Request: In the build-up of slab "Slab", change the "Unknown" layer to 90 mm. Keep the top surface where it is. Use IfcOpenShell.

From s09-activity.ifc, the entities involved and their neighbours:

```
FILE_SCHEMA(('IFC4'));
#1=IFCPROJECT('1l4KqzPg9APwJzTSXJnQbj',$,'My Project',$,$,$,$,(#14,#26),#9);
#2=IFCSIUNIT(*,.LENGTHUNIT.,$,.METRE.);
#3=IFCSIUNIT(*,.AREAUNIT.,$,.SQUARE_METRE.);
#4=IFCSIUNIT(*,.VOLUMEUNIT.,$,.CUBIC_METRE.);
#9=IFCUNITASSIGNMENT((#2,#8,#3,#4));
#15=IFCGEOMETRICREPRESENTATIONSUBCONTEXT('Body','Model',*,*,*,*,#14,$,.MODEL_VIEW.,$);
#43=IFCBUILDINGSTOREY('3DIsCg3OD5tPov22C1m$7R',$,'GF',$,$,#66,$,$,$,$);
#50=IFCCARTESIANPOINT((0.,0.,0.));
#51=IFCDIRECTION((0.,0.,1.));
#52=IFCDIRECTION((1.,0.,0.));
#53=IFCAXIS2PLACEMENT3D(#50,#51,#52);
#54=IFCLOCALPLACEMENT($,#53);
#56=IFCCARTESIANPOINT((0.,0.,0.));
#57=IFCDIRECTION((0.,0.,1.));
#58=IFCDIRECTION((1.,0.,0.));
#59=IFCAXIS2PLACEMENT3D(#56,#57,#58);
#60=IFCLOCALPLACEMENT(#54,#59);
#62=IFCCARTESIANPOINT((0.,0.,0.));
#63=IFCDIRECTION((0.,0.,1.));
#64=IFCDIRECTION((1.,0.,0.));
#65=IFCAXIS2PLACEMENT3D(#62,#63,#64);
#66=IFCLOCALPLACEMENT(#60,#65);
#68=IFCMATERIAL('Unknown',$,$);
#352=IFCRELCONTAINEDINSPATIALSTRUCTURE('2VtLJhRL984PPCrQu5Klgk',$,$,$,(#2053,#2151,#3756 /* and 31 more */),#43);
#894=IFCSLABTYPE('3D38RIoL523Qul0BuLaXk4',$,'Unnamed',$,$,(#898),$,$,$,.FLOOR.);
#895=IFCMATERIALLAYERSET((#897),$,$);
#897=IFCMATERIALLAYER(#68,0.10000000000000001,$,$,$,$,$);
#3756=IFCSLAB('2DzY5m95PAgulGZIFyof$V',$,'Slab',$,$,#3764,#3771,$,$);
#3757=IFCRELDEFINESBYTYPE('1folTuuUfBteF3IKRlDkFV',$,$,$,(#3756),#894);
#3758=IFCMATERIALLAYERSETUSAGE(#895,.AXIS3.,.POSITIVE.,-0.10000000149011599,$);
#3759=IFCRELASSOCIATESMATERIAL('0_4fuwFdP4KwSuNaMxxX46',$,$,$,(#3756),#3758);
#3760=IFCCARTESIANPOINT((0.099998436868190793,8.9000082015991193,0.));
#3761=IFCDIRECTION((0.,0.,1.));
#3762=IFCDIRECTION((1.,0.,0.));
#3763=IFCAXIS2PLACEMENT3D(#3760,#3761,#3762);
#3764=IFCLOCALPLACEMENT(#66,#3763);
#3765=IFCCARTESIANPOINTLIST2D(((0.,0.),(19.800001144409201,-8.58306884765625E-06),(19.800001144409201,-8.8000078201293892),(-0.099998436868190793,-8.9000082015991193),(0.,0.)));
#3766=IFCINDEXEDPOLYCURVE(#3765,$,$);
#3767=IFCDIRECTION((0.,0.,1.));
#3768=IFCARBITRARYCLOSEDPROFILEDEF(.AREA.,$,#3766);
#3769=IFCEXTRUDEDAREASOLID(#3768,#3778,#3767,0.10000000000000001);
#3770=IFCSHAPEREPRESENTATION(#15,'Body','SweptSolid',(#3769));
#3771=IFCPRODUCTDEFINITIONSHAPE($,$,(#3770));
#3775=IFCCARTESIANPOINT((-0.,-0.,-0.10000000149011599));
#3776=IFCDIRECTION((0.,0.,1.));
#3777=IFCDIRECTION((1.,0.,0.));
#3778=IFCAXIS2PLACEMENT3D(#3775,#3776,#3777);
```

```python
import ifcopenshell
import ifcopenshell.util.element
import ifcopenshell.util.representation

model = ifcopenshell.open("s09-activity.ifc")

layer_set = model.by_id(895)
layer = next(l for l in layer_set.MaterialLayers if l.Material and l.Material.Name == "Unknown")
change = 0.09 - layer.LayerThickness
layer.LayerThickness += change

# Geometry does not follow the layer set by itself.
slabs = [e for e in ifcopenshell.util.element.get_elements_by_material(model, layer_set) if e.is_a("IfcSlab")]
for slab in sorted(slabs, key=lambda e: e.id()):
    body = ifcopenshell.util.representation.get_representation(slab, "Model", "Body")
    solid = body.Items[0]
    old_depth = solid.Depth
    solid.Depth += change
    # Extruded upwards: lower the start of the extrusion so the top stays.
    x, y, z = solid.Position.Location.Coordinates
    solid.Position.Location = model.createIfcCartesianPoint((x, y, z - change))
    print(slab.id(), f"{old_depth:g} -> {solid.Depth:g}")

# The layers are counted up from the underside, which has moved.
for usage in {ifcopenshell.util.element.get_material(slab) for slab in slabs}:
    usage.OffsetFromReferenceLine -= change

model.write("s09-activity_rev.ifc")
```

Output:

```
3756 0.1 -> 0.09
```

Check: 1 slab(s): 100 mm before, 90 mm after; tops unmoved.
